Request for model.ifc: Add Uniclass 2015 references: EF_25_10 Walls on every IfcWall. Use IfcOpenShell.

First a look at what the model holds.

```python
import ifcopenshell

model = ifcopenshell.open("model.ifc")
print(model.schema)
print("classifications:", [c.Name for c in model.by_type("IfcClassification")])
for ifc_class in ("IfcDoor", "IfcRoof", "IfcStair", "IfcWall", "IfcWindow"):
    print(ifc_class, len(model.by_type(ifc_class)))
```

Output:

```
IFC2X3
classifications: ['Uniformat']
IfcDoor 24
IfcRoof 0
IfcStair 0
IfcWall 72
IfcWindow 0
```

```python
import ifcopenshell
import ifcopenshell.api.classification

model = ifcopenshell.open("model.ifc")

# IFC2X3 requires Source and Edition and has no link from the project to the system.
system = model.create_entity("IfcClassification", Source="NBS", Edition="2015", Name="Uniclass 2015")

codes = {
    "IfcWall": ("EF_25_10", "Walls"),
}
for ifc_class, (code, name) in codes.items():
    products = model.by_type(ifc_class)
    ifcopenshell.api.classification.add_reference(
        model, products=products, classification=system, identification=code, name=name
    )
    print(code, len(products))

model.write("model-out.ifc")
```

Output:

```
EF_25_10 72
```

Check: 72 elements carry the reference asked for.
